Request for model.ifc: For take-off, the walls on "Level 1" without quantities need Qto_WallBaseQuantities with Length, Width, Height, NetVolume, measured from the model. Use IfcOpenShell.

First a look at what the model holds.

```python
import ifcopenshell
import ifcopenshell.util.element
import ifcopenshell.util.unit

model = ifcopenshell.open("model.ifc")
print(model.schema)
for unit_type in ("LENGTHUNIT", "AREAUNIT", "VOLUMEUNIT"):
    print(unit_type, ifcopenshell.util.unit.calculate_unit_scale(model, unit_type))
storey = next(s for s in model.by_type("IfcBuildingStorey") if s.Name == "Level 1")
walls = [e for e in ifcopenshell.util.element.get_decomposition(storey) if e.is_a("IfcWall")]
for e in sorted(walls, key=lambda e: e.id()):
    print(e.id(), e.is_a(), e.Name, list(ifcopenshell.util.element.get_psets(e, qtos_only=True)), sep=" | ")
```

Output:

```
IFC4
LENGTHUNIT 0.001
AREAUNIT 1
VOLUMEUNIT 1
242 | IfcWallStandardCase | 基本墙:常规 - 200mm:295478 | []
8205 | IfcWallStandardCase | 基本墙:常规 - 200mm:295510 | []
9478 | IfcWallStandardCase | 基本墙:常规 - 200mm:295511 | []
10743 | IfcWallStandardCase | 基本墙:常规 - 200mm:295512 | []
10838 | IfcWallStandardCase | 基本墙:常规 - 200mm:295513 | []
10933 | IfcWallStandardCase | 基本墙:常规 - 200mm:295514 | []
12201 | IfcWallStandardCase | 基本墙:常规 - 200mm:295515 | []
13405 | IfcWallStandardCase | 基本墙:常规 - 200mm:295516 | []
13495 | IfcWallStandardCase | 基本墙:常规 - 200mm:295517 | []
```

```python
import ifcopenshell
import ifcopenshell.api.pset
import ifcopenshell.geom
import ifcopenshell.util.element
import ifcopenshell.util.shape
import ifcopenshell.util.unit

model = ifcopenshell.open("model.ifc")
unit_scale = ifcopenshell.util.unit.calculate_unit_scale(model)
volume_scale = ifcopenshell.util.unit.calculate_unit_scale(model, "VOLUMEUNIT")
settings = ifcopenshell.geom.settings()

storey = next(s for s in model.by_type("IfcBuildingStorey") if s.Name == "Level 1")
walls = [e for e in ifcopenshell.util.element.get_decomposition(storey) if e.is_a("IfcWall")]

for e in sorted(walls, key=lambda e: e.id()):
    if ifcopenshell.util.element.get_psets(e, qtos_only=True, should_inherit=False):
        continue
    # Geometry comes back in metres, in the element's own axes.
    shape = ifcopenshell.geom.create_shape(settings, e)
    values = {
        "Length": ifcopenshell.util.shape.get_x(shape.geometry) / unit_scale,
        "Width": ifcopenshell.util.shape.get_y(shape.geometry) / unit_scale,
        "Height": ifcopenshell.util.shape.get_z(shape.geometry) / unit_scale,
        "NetVolume": ifcopenshell.util.shape.get_volume(shape.geometry) / volume_scale,
    }
    qto = ifcopenshell.api.pset.add_qto(model, product=e, name="Qto_WallBaseQuantities")
    ifcopenshell.api.pset.edit_qto(model, qto=qto, properties=values)
    print(e.id(), {k: round(v, 3) for k, v in values.items()})

model.write("model_v2.ifc")
```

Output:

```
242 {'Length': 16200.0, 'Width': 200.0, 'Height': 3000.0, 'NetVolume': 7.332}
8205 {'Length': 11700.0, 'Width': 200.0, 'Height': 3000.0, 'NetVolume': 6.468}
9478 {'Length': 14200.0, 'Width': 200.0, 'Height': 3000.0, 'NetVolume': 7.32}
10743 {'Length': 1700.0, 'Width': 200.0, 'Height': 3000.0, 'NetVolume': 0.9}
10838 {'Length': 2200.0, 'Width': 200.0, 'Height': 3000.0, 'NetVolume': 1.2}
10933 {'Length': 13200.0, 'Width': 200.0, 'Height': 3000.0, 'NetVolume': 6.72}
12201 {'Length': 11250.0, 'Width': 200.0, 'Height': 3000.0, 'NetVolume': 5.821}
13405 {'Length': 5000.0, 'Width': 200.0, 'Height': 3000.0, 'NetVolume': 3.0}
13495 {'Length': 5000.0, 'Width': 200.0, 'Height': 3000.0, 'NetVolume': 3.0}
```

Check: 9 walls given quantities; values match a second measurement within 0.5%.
